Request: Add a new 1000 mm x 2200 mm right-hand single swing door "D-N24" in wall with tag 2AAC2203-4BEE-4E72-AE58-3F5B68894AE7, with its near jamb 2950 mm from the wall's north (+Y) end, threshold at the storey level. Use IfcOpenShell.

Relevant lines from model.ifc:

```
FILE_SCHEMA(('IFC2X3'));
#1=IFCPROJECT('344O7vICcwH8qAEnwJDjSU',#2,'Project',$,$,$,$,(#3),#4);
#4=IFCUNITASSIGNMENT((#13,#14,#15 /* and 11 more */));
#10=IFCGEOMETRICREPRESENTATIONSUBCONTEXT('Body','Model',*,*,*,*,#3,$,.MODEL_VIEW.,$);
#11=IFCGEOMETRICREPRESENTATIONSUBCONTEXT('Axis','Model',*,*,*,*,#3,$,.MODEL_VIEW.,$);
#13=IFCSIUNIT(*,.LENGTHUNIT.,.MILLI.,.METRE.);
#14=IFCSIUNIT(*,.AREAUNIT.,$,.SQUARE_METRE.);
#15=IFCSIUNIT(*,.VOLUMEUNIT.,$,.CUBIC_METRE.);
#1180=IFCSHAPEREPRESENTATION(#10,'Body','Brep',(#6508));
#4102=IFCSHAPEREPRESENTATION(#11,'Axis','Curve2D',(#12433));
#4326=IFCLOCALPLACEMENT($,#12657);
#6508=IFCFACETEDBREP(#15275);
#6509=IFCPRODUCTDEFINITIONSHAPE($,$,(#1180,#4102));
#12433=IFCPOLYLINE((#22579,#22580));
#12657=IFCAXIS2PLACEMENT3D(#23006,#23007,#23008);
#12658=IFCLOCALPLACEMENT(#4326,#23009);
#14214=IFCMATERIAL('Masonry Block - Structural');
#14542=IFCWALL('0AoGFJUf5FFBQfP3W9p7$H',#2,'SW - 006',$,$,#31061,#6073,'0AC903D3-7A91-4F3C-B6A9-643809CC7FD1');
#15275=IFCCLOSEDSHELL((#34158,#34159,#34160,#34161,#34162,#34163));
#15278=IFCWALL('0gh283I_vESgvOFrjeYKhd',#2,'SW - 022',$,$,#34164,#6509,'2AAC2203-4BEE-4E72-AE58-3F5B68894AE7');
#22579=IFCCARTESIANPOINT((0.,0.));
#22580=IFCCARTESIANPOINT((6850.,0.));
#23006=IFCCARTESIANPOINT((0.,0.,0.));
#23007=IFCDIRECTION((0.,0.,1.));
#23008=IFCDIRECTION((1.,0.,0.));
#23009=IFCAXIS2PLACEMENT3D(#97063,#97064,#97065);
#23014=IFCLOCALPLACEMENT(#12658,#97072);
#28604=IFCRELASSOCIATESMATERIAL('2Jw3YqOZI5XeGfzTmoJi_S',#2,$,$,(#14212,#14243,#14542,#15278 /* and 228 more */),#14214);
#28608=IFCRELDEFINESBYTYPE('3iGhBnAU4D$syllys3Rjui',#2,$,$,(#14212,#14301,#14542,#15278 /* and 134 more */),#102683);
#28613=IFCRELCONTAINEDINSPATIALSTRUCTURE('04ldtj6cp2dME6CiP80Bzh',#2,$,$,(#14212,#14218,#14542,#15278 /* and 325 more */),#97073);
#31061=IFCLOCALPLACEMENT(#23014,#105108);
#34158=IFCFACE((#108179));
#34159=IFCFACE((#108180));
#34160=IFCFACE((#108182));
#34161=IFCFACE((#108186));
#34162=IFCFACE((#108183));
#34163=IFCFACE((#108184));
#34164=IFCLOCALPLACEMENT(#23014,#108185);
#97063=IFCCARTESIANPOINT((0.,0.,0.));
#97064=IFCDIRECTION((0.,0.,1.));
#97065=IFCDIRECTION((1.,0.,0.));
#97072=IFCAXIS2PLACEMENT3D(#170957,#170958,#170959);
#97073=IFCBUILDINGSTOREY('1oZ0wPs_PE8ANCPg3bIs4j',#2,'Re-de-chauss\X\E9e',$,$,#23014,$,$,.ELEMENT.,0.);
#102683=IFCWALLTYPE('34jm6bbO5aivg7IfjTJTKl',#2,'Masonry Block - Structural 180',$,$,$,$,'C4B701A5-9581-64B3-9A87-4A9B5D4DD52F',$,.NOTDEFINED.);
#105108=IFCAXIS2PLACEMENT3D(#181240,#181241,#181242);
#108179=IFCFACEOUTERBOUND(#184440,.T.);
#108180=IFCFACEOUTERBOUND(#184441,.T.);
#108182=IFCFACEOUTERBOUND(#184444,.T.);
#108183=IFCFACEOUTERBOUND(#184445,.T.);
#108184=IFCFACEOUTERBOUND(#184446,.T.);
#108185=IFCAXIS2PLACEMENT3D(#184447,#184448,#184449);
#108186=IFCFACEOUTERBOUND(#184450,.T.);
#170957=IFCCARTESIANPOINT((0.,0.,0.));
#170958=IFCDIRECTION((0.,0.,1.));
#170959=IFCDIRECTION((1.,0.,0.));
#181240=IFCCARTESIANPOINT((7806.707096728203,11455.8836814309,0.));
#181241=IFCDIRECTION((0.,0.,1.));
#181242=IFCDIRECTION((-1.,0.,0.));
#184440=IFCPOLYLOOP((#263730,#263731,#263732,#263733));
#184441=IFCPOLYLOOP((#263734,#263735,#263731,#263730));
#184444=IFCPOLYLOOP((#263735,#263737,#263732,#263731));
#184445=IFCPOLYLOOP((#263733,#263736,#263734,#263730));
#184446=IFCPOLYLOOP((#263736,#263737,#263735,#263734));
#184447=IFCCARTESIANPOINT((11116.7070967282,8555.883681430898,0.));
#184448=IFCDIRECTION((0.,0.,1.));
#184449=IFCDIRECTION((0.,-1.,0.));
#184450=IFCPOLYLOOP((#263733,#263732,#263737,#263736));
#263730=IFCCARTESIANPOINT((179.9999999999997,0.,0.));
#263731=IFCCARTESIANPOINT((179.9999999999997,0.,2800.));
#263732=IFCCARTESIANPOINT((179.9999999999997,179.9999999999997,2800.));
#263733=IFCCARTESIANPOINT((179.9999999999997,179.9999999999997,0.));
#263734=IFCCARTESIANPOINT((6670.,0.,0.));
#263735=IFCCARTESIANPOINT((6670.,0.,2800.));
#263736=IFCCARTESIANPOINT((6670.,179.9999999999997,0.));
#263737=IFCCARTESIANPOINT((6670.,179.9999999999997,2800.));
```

```python
import numpy as np
import ifcopenshell
import ifcopenshell.api.feature
import ifcopenshell.api.geometry
import ifcopenshell.api.root
import ifcopenshell.api.spatial
import ifcopenshell.api.type
import ifcopenshell.geom
import ifcopenshell.util.element
import ifcopenshell.util.placement
import ifcopenshell.util.representation
import ifcopenshell.util.shape
import ifcopenshell.util.unit

model = ifcopenshell.open("model.ifc")
unit_scale = ifcopenshell.util.unit.calculate_unit_scale(model)
settings = ifcopenshell.geom.settings()


def volume(element):
    """Net volume in cubic metres, openings subtracted."""
    shape = ifcopenshell.geom.create_shape(settings, element)
    return ifcopenshell.util.shape.get_volume(shape.geometry)


wall = model.by_guid("0gh283I_vESgvOFrjeYKhd")
storey = ifcopenshell.util.element.get_container(wall, ifc_class="IfcBuildingStorey")
context = ifcopenshell.util.representation.get_context(model, "Model", "Body", "MODEL_VIEW")
before = volume(wall)

width, height, from_end, sill = 1, 2.2, 2.95, 0.0  # metres

# The wall runs along its own X axis, and the end named is its -X end.
wall_shape = ifcopenshell.geom.create_shape(settings, wall)
x, y, z = ifcopenshell.util.shape.get_vertices(wall_shape.geometry).T
start = x.min() + from_end
face, thickness = float(y.min()), float(y.max() - y.min())
wall_matrix = ifcopenshell.util.placement.get_local_placement(wall.ObjectPlacement)
level = ifcopenshell.util.placement.get_local_placement(storey.ObjectPlacement)[2, 3]


def in_wall(x, y):
    """Placement at x, y metres in the wall's axes, at sill height."""
    matrix = wall_matrix.copy()
    matrix[:, 3] = wall_matrix @ np.array([x / unit_scale, y / unit_scale, 0.0, 1.0])
    matrix[2, 3] = level + sill / unit_scale
    return matrix


# Opening: a box that overshoots both wall faces by 50 mm.
opening = ifcopenshell.api.root.create_entity(model, ifc_class="IfcOpeningElement")
box = ifcopenshell.api.geometry.add_wall_representation(
    model, context=context, length=width, height=height, thickness=thickness + 0.1
)
ifcopenshell.api.geometry.assign_representation(model, product=opening, representation=box)
ifcopenshell.api.geometry.edit_object_placement(model, product=opening, matrix=in_wall(start, face - 0.05), is_si=False)
ifcopenshell.api.feature.add_feature(model, feature=opening, element=wall)

door = ifcopenshell.api.root.create_entity(model, ifc_class="IfcDoor", name="D-N24")
door.OverallWidth, door.OverallHeight = width / unit_scale, height / unit_scale
body = ifcopenshell.api.geometry.add_door_representation(
    model,
    context=context,
    overall_width=door.OverallWidth,
    overall_height=door.OverallHeight,
    operation_type="SINGLE_SWING_RIGHT",
    lining_properties={"LiningDepth": thickness / unit_scale, "ThresholdDepth": thickness / unit_scale},
)
ifcopenshell.api.geometry.assign_representation(model, product=door, representation=body)
ifcopenshell.api.spatial.assign_container(model, products=[door], relating_structure=storey)
fills = ifcopenshell.api.feature.add_filling(model, opening=opening, element=door)
fills.OwnerHistory = door.OwnerHistory  # required in IFC2X3

# IFC2X3 keeps the operation on the door style.
style = ifcopenshell.api.root.create_entity(model, ifc_class="IfcDoorStyle", name="D-N24")
style.OperationType, style.ConstructionType = "SINGLE_SWING_RIGHT", "NOTDEFINED"
style.ParameterTakesPrecedence = style.Sizeable = False
ifcopenshell.api.type.assign_type(model, related_objects=[door], relating_type=style)

# The lining spans the wall, so the door starts at the wall face.
ifcopenshell.api.geometry.edit_object_placement(model, product=door, matrix=in_wall(start, face), is_si=False)

after = volume(wall)

print(f"wall volume {before:.3f} -> {after:.3f} m3")

model.write("model_edited.ifc")
```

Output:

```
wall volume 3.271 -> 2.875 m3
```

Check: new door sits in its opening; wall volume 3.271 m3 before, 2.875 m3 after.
